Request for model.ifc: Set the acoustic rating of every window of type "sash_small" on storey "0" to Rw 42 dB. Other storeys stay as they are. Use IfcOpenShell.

First a look at what the model holds.

```python
import ifcopenshell
import ifcopenshell.util.element

model = ifcopenshell.open("model.ifc")
print(model.schema)
storey = next(s for s in model.by_type("IfcBuildingStorey") if s.Name == "0")
windows = [e for e in ifcopenshell.util.element.get_decomposition(storey) if e.is_a("IfcWindow")]
seen = {}
for e in windows:
    element_type = ifcopenshell.util.element.get_type(e)
    key = (element_type.Name if element_type != e and element_type else None, ifcopenshell.util.element.get_pset(e, "Pset_WindowCommon", "AcousticRating"))
    seen[key] = seen.get(key, 0) + 1
for (name, value), count in sorted(seen.items(), key=str):
    print(count, "x", name, "|", value)
```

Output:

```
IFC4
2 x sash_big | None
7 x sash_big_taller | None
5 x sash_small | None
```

```python
import ifcopenshell
import ifcopenshell.api.pset
import ifcopenshell.util.element

model = ifcopenshell.open("model.ifc")

storey = next(s for s in model.by_type("IfcBuildingStorey") if s.Name == "0")
windows = [e for e in ifcopenshell.util.element.get_decomposition(storey) if e.is_a("IfcWindow")]

count = 0
for e in windows:
    element_type = ifcopenshell.util.element.get_type(e)
    if element_type in (None, e) or element_type.Name != "sash_small":
        continue
    # add_pset returns the element's existing set when there is one.
    pset = ifcopenshell.api.pset.add_pset(model, product=e, name="Pset_WindowCommon")
    ifcopenshell.api.pset.edit_pset(model, pset=pset, properties={"AcousticRating": "Rw 42 dB"})
    count += 1

print(count, "windows updated")

model.write("model-out.ifc")
```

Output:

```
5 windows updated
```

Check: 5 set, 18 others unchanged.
